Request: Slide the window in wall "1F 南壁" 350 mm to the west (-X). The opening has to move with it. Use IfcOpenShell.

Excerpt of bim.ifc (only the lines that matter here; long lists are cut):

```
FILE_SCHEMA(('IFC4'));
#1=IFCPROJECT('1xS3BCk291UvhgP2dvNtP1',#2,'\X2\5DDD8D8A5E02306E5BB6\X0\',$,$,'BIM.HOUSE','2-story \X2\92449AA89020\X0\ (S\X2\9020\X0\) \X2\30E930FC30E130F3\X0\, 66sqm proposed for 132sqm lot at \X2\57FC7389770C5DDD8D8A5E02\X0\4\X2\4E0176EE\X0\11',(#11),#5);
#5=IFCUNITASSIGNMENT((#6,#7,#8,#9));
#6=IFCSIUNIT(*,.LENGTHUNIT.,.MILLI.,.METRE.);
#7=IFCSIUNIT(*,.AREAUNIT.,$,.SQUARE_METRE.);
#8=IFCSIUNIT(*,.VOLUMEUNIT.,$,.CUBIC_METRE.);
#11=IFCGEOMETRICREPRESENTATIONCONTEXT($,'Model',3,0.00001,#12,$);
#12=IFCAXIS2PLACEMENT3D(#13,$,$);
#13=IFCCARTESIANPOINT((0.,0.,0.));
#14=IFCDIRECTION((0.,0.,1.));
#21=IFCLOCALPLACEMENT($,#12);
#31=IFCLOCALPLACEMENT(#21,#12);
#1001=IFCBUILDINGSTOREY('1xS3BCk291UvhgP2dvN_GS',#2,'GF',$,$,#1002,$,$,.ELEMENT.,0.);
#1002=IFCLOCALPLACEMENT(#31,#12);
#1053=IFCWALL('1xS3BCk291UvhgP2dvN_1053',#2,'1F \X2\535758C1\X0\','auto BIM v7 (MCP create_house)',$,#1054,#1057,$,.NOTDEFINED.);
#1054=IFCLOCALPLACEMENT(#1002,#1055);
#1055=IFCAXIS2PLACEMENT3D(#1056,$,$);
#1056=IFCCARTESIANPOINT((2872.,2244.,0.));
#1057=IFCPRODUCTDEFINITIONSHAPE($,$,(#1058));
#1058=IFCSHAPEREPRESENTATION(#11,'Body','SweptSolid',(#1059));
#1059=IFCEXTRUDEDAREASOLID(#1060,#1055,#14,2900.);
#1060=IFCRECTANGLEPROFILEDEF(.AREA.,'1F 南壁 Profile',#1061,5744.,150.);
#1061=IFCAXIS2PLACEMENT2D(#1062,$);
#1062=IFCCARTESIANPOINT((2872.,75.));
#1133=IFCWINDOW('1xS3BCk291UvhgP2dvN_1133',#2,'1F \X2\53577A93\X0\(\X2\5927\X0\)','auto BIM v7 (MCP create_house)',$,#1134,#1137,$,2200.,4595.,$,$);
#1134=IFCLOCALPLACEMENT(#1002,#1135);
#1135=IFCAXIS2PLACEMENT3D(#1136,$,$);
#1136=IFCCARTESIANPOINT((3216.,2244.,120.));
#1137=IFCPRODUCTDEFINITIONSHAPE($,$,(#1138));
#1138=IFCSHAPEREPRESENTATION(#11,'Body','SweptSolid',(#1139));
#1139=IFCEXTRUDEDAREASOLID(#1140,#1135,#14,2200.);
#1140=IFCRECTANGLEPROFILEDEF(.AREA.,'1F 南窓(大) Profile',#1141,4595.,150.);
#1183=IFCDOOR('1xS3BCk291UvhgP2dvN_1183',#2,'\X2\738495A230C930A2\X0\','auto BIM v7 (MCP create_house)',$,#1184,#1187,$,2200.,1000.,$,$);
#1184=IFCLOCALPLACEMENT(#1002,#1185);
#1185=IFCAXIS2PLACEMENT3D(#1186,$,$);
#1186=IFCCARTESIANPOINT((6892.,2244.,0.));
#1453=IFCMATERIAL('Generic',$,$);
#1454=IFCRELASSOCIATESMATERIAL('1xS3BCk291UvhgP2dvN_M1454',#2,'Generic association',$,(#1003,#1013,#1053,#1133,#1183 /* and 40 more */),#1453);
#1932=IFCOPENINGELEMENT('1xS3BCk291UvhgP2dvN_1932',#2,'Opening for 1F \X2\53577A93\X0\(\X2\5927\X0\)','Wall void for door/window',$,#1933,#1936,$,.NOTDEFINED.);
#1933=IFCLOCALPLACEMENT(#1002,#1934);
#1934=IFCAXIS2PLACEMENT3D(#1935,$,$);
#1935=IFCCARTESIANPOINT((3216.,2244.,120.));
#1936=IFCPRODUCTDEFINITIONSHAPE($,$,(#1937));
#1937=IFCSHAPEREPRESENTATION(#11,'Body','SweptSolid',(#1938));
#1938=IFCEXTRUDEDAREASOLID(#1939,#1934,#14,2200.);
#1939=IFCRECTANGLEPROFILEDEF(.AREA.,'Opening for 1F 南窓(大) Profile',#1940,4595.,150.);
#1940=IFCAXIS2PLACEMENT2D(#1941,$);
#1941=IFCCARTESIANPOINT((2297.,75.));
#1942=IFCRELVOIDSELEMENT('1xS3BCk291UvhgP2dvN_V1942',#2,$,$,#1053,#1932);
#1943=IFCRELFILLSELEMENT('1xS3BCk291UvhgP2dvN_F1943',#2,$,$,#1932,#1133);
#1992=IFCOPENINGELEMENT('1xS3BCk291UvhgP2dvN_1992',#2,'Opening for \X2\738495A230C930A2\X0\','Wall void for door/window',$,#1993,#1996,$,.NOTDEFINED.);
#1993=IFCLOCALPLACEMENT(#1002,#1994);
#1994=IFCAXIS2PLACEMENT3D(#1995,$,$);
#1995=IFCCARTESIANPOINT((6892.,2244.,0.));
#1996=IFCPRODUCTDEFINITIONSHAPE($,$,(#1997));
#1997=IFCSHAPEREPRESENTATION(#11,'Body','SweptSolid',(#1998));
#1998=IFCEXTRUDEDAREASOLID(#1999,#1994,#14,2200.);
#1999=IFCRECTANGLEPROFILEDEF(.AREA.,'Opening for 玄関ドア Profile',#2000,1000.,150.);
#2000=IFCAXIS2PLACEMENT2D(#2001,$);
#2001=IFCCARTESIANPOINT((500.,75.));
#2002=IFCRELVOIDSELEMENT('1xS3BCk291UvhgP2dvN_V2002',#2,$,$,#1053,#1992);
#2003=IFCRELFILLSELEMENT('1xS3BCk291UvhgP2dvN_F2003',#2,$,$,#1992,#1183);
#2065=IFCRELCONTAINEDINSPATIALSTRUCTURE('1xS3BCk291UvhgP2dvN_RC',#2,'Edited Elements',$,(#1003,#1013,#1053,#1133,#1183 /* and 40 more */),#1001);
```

```python
import ifcopenshell
import ifcopenshell.api.geometry
import ifcopenshell.util.placement

model = ifcopenshell.open("bim.ifc")

window = model.by_guid("1xS3BCk291UvhgP2dvN_1133")
opening = window.FillsVoids[0].RelatingOpeningElement
wall = opening.VoidsElements[0].RelatingBuildingElement

wall_matrix = ifcopenshell.util.placement.get_local_placement(wall.ObjectPlacement)
shift = wall_matrix[:3, 0] * -350.0
before = ifcopenshell.util.placement.get_local_placement(window.ObjectPlacement)[:3, 3].copy()

# The window is not placed relative to its opening, so move both.
for product in (opening, window):
    matrix = ifcopenshell.util.placement.get_local_placement(product.ObjectPlacement)
    matrix[:3, 3] += shift
    ifcopenshell.api.geometry.edit_object_placement(model, product=product, matrix=matrix, is_si=False)

after = ifcopenshell.util.placement.get_local_placement(window.ObjectPlacement)[:3, 3]
print("window moved by", (after - before).round(3) + 0.0)

model.write("bim-out.ifc")
```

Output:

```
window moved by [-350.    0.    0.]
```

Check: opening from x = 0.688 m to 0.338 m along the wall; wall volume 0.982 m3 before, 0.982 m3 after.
